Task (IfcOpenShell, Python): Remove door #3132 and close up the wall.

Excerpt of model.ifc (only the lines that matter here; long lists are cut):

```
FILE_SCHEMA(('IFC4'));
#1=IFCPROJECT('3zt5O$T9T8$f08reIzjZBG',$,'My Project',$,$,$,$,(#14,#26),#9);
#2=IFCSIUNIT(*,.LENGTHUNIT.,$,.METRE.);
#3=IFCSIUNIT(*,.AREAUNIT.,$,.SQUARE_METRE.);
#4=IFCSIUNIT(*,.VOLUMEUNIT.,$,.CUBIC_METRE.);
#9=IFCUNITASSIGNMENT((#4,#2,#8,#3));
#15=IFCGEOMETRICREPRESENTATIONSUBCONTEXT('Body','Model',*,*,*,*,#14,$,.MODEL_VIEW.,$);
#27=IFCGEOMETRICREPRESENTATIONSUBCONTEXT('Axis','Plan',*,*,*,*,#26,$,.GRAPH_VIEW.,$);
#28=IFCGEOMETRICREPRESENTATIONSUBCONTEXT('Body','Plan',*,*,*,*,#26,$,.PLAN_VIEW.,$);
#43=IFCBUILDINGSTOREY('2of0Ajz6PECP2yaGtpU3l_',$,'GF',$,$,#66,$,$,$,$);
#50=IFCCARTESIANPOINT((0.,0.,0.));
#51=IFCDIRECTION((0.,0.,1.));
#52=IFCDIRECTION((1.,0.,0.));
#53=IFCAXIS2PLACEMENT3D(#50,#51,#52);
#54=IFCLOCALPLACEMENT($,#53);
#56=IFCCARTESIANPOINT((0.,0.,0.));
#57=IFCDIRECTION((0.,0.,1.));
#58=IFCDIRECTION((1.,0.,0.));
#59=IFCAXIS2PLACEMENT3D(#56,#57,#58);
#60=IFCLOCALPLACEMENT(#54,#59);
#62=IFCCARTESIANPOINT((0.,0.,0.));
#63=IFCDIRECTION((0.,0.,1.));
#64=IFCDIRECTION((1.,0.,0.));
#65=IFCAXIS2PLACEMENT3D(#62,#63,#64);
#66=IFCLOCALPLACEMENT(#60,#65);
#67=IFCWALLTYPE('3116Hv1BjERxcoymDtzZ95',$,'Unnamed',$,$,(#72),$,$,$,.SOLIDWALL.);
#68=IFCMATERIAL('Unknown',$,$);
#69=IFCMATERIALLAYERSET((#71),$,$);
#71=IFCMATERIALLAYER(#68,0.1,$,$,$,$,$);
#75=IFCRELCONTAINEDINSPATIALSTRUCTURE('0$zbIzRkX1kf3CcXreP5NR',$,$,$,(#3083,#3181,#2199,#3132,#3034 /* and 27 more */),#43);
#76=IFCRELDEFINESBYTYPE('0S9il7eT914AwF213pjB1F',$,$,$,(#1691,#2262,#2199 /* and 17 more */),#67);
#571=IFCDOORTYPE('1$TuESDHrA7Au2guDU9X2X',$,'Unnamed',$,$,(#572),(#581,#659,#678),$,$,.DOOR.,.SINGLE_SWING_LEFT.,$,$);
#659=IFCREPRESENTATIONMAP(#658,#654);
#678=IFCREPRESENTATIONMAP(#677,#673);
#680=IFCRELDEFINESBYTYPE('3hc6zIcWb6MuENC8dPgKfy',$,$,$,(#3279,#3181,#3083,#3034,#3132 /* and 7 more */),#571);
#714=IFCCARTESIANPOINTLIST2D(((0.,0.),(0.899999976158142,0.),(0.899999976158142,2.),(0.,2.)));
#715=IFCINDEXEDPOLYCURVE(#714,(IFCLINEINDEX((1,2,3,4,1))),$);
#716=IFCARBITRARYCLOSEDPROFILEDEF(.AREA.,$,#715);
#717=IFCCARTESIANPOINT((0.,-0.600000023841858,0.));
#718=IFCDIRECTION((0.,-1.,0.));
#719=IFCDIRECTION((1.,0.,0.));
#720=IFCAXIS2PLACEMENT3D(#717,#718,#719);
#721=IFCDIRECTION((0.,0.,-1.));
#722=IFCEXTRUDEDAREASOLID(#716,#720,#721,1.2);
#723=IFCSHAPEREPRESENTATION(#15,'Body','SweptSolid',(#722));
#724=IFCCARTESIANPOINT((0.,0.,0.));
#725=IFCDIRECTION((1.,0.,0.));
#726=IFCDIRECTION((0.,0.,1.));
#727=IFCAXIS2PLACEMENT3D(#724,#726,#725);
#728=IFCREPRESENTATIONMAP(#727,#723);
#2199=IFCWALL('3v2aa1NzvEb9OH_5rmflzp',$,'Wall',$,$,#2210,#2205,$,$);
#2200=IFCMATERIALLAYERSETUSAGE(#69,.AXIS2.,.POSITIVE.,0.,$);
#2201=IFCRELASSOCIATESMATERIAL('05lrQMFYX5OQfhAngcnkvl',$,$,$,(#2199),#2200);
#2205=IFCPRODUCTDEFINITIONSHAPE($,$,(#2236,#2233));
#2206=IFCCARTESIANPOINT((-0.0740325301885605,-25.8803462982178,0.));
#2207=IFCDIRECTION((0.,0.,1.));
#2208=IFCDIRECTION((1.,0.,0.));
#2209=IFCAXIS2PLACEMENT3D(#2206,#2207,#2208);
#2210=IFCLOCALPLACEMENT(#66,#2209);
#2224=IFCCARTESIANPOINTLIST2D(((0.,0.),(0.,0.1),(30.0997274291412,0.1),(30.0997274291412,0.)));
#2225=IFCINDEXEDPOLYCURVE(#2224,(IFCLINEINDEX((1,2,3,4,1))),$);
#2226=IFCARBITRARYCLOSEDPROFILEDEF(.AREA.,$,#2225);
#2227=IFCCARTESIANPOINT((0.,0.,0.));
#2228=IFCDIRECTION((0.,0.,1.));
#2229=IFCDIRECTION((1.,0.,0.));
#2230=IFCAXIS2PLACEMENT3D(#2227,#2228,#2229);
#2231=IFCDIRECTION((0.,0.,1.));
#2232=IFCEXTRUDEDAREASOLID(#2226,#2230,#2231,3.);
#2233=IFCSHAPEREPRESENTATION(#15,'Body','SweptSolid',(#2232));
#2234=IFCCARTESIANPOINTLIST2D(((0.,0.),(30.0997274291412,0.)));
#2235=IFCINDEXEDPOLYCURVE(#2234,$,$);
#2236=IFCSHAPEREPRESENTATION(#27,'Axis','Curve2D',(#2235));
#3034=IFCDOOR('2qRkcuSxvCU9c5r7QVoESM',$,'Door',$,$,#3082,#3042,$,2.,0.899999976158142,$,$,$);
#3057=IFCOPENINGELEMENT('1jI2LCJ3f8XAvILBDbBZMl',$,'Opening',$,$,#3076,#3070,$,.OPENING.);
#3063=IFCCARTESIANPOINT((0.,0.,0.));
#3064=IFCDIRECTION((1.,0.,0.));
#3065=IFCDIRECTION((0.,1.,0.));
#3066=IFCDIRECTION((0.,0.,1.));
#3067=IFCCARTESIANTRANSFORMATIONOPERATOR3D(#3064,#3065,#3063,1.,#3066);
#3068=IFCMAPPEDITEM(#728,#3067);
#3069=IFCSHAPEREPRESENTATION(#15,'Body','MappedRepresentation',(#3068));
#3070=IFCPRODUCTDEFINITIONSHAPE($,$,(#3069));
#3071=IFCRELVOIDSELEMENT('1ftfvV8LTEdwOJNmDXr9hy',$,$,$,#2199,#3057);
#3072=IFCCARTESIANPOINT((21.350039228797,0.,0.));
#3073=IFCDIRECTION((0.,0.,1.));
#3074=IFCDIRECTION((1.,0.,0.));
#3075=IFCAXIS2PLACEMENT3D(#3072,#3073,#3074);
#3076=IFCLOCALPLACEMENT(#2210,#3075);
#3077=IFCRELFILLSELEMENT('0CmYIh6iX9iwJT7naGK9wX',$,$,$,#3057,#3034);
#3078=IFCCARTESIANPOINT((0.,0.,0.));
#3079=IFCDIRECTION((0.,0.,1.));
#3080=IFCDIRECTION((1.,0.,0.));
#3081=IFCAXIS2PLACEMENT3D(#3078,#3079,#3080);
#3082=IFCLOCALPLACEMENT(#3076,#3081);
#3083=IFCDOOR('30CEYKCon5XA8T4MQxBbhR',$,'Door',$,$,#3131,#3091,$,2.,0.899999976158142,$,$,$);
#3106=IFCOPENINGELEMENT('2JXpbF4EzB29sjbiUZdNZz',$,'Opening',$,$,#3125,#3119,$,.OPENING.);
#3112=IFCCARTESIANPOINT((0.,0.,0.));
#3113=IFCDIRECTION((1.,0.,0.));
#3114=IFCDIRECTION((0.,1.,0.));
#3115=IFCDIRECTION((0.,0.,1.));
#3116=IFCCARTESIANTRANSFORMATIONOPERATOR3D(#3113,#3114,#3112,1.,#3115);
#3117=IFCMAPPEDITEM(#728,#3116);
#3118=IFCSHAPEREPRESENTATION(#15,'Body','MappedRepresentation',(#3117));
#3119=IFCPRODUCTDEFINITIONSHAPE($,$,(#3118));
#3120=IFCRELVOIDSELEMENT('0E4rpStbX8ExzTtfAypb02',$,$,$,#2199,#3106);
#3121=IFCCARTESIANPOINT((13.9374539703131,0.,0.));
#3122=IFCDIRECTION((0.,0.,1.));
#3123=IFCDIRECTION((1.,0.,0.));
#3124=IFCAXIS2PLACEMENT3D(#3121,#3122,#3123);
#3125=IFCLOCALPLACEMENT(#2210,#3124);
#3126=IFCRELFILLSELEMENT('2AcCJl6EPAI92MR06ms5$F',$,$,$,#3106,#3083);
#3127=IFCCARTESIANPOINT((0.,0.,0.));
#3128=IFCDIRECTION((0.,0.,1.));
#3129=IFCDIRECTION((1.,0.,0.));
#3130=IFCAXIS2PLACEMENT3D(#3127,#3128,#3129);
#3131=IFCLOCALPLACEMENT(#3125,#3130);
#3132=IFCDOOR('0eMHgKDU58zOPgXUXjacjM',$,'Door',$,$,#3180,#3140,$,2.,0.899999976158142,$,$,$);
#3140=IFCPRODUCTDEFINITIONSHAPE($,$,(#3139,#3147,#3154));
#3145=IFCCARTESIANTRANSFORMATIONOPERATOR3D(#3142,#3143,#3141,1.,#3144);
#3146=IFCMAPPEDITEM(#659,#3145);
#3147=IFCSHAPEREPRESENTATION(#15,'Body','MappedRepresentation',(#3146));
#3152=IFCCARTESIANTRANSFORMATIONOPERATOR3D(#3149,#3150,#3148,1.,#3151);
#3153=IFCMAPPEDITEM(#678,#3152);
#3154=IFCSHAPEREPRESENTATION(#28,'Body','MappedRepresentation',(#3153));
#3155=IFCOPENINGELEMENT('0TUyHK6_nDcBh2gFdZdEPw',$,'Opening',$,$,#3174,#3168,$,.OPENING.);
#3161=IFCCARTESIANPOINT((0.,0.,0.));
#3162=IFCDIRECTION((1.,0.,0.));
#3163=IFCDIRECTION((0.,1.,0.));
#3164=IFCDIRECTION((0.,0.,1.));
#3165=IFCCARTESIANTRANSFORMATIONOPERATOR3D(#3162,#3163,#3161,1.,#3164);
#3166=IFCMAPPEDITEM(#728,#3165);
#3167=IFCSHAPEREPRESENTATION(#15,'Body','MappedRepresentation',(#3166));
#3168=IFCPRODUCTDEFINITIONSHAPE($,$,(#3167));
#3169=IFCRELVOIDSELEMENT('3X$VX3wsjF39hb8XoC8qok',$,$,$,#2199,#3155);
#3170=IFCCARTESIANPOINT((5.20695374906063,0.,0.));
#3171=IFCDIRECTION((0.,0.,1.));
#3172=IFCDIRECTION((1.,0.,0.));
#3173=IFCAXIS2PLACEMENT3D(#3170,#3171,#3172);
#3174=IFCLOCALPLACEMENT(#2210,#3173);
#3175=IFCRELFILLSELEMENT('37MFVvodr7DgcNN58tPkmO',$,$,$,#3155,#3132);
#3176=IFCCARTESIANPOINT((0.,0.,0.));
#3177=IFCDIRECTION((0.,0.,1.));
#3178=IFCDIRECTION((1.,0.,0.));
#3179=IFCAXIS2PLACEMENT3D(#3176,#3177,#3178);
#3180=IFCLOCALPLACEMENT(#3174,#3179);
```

```python
import ifcopenshell
import ifcopenshell.api.feature
import ifcopenshell.api.root
import ifcopenshell.geom
import ifcopenshell.util.shape

model = ifcopenshell.open("model.ifc")
settings = ifcopenshell.geom.settings()


def volume(element):
    """Net volume in cubic metres, openings subtracted."""
    shape = ifcopenshell.geom.create_shape(settings, element)
    return ifcopenshell.util.shape.get_volume(shape.geometry)


door = model.by_id(3132)
opening = door.FillsVoids[0].RelatingOpeningElement
wall = opening.VoidsElements[0].RelatingBuildingElement
before = volume(wall)

ifcopenshell.api.root.remove_product(model, product=door)
ifcopenshell.api.feature.remove_feature(model, feature=opening)

after = volume(wall)

print(f"wall volume {before:.3f} -> {after:.3f} m3")

model.write("model_edited.ifc")
```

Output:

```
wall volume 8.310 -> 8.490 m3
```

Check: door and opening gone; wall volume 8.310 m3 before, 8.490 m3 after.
